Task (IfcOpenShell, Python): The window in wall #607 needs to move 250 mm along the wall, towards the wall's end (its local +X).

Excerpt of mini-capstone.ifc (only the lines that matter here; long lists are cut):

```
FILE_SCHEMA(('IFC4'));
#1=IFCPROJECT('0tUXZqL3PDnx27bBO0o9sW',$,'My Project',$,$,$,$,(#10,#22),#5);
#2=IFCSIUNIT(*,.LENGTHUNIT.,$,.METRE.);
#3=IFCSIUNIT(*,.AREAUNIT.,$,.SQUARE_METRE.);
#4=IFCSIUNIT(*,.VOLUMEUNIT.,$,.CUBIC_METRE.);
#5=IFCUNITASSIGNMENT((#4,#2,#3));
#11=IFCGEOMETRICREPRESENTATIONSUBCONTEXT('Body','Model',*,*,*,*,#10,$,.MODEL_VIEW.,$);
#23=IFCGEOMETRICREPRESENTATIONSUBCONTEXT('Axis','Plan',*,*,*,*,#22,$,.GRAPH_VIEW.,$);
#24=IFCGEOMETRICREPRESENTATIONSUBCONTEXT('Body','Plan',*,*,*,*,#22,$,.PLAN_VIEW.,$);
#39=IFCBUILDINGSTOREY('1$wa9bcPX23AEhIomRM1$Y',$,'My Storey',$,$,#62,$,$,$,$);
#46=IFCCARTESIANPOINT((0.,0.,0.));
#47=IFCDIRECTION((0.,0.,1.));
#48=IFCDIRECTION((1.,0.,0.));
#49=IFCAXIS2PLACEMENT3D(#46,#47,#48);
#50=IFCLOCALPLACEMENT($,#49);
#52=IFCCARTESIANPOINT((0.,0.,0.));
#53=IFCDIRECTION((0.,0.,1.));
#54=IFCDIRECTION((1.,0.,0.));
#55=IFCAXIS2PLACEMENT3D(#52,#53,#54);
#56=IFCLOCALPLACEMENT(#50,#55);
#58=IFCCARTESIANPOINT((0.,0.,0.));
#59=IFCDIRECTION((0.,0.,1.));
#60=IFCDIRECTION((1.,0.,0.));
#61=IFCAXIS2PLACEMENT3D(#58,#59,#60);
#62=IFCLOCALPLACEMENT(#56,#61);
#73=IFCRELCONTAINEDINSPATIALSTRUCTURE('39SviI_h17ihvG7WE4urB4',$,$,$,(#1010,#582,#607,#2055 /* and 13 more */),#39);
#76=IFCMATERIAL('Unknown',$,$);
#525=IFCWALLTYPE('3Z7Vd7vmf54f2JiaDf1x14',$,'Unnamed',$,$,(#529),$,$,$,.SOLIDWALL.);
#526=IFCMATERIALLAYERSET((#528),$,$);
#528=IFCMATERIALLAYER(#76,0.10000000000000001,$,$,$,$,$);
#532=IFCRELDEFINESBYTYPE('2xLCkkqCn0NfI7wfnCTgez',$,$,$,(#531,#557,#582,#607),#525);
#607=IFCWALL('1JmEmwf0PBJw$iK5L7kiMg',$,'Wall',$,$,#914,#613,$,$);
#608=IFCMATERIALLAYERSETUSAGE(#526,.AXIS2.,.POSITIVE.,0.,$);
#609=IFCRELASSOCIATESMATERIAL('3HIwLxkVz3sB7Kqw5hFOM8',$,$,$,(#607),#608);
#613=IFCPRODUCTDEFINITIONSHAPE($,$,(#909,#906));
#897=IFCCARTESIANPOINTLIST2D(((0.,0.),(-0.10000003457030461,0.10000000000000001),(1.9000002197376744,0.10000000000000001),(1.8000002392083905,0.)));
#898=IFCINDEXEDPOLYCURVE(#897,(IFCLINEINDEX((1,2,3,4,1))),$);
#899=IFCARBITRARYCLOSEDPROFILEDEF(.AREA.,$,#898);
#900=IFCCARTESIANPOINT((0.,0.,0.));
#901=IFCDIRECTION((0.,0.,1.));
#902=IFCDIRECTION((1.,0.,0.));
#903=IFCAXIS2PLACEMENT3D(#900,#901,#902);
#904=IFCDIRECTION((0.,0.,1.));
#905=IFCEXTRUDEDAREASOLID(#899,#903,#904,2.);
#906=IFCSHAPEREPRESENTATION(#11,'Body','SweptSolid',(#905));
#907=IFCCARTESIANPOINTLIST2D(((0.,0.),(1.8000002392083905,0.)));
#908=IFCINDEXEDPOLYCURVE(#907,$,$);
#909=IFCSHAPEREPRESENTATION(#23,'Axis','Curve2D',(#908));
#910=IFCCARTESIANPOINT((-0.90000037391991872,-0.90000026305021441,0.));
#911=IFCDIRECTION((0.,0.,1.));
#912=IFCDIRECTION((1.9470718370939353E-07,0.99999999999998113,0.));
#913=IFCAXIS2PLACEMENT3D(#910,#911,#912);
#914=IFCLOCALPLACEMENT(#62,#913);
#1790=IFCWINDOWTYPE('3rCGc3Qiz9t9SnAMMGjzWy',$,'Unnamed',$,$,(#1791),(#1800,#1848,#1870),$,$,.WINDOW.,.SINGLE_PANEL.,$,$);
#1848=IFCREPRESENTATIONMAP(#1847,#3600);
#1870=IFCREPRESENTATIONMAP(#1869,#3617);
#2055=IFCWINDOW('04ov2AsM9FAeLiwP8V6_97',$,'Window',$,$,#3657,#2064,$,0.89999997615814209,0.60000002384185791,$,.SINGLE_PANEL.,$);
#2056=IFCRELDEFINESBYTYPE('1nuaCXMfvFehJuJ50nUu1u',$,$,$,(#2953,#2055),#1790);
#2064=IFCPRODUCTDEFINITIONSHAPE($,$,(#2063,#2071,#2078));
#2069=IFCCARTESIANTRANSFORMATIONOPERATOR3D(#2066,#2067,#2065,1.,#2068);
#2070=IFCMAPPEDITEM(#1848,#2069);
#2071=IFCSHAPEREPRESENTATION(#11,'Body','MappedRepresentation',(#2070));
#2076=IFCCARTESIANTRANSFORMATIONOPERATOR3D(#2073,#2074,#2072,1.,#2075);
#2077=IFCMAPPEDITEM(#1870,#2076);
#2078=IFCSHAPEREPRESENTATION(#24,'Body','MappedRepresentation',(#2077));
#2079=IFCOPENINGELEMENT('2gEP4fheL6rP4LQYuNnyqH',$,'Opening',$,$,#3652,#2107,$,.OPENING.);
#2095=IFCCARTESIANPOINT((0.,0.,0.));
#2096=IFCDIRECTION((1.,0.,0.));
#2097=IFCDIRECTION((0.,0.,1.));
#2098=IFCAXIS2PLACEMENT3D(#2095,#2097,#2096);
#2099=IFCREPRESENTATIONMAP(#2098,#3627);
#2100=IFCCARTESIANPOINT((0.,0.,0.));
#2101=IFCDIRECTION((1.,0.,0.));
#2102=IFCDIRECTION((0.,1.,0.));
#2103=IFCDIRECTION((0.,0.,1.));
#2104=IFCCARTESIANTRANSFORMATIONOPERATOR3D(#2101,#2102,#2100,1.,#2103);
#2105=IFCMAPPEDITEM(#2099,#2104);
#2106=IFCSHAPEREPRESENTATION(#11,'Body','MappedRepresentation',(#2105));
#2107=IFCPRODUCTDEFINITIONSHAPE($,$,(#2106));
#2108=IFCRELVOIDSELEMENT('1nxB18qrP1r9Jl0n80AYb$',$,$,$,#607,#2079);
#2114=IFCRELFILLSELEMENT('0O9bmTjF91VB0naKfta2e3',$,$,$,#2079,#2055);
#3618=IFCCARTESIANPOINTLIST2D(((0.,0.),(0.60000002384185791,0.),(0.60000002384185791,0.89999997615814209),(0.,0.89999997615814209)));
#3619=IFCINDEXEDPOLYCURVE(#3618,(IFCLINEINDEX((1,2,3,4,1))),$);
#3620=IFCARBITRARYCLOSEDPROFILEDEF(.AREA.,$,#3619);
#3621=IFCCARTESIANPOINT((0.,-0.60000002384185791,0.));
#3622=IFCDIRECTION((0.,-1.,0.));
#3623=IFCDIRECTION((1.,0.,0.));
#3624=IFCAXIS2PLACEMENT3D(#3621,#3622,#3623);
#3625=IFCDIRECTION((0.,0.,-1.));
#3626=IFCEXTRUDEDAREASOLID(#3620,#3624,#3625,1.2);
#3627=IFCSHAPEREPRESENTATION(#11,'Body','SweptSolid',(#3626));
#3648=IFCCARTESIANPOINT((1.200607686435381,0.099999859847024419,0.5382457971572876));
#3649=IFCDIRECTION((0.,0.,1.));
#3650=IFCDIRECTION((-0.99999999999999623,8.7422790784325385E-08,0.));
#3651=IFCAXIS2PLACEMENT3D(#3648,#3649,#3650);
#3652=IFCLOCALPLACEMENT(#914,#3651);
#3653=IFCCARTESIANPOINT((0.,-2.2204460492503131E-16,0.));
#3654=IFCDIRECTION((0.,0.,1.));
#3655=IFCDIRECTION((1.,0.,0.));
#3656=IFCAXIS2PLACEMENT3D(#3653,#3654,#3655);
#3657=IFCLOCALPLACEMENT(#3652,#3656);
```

```python
import ifcopenshell
import ifcopenshell.api.geometry
import ifcopenshell.util.placement
import ifcopenshell.util.unit

model = ifcopenshell.open("mini-capstone.ifc")
unit_scale = ifcopenshell.util.unit.calculate_unit_scale(model)

window = model.by_id(2055)
opening = window.FillsVoids[0].RelatingOpeningElement
wall = opening.VoidsElements[0].RelatingBuildingElement

wall_matrix = ifcopenshell.util.placement.get_local_placement(wall.ObjectPlacement)
shift = wall_matrix[:3, 0] * 0.25 / unit_scale
before = ifcopenshell.util.placement.get_local_placement(window.ObjectPlacement)[:3, 3].copy()

# The window is placed relative to its opening, so it follows when the opening moves.
matrix = ifcopenshell.util.placement.get_local_placement(opening.ObjectPlacement)
matrix[:3, 3] += shift
ifcopenshell.api.geometry.edit_object_placement(
    model, product=opening, matrix=matrix, is_si=False, should_transform_children=True
)

after = ifcopenshell.util.placement.get_local_placement(window.ObjectPlacement)[:3, 3]
print("window moved by", (after - before).round(3) + 0.0)

model.write("mini-capstone_updated.ifc")
```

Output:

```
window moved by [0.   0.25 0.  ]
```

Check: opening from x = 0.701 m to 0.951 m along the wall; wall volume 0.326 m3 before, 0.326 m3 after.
